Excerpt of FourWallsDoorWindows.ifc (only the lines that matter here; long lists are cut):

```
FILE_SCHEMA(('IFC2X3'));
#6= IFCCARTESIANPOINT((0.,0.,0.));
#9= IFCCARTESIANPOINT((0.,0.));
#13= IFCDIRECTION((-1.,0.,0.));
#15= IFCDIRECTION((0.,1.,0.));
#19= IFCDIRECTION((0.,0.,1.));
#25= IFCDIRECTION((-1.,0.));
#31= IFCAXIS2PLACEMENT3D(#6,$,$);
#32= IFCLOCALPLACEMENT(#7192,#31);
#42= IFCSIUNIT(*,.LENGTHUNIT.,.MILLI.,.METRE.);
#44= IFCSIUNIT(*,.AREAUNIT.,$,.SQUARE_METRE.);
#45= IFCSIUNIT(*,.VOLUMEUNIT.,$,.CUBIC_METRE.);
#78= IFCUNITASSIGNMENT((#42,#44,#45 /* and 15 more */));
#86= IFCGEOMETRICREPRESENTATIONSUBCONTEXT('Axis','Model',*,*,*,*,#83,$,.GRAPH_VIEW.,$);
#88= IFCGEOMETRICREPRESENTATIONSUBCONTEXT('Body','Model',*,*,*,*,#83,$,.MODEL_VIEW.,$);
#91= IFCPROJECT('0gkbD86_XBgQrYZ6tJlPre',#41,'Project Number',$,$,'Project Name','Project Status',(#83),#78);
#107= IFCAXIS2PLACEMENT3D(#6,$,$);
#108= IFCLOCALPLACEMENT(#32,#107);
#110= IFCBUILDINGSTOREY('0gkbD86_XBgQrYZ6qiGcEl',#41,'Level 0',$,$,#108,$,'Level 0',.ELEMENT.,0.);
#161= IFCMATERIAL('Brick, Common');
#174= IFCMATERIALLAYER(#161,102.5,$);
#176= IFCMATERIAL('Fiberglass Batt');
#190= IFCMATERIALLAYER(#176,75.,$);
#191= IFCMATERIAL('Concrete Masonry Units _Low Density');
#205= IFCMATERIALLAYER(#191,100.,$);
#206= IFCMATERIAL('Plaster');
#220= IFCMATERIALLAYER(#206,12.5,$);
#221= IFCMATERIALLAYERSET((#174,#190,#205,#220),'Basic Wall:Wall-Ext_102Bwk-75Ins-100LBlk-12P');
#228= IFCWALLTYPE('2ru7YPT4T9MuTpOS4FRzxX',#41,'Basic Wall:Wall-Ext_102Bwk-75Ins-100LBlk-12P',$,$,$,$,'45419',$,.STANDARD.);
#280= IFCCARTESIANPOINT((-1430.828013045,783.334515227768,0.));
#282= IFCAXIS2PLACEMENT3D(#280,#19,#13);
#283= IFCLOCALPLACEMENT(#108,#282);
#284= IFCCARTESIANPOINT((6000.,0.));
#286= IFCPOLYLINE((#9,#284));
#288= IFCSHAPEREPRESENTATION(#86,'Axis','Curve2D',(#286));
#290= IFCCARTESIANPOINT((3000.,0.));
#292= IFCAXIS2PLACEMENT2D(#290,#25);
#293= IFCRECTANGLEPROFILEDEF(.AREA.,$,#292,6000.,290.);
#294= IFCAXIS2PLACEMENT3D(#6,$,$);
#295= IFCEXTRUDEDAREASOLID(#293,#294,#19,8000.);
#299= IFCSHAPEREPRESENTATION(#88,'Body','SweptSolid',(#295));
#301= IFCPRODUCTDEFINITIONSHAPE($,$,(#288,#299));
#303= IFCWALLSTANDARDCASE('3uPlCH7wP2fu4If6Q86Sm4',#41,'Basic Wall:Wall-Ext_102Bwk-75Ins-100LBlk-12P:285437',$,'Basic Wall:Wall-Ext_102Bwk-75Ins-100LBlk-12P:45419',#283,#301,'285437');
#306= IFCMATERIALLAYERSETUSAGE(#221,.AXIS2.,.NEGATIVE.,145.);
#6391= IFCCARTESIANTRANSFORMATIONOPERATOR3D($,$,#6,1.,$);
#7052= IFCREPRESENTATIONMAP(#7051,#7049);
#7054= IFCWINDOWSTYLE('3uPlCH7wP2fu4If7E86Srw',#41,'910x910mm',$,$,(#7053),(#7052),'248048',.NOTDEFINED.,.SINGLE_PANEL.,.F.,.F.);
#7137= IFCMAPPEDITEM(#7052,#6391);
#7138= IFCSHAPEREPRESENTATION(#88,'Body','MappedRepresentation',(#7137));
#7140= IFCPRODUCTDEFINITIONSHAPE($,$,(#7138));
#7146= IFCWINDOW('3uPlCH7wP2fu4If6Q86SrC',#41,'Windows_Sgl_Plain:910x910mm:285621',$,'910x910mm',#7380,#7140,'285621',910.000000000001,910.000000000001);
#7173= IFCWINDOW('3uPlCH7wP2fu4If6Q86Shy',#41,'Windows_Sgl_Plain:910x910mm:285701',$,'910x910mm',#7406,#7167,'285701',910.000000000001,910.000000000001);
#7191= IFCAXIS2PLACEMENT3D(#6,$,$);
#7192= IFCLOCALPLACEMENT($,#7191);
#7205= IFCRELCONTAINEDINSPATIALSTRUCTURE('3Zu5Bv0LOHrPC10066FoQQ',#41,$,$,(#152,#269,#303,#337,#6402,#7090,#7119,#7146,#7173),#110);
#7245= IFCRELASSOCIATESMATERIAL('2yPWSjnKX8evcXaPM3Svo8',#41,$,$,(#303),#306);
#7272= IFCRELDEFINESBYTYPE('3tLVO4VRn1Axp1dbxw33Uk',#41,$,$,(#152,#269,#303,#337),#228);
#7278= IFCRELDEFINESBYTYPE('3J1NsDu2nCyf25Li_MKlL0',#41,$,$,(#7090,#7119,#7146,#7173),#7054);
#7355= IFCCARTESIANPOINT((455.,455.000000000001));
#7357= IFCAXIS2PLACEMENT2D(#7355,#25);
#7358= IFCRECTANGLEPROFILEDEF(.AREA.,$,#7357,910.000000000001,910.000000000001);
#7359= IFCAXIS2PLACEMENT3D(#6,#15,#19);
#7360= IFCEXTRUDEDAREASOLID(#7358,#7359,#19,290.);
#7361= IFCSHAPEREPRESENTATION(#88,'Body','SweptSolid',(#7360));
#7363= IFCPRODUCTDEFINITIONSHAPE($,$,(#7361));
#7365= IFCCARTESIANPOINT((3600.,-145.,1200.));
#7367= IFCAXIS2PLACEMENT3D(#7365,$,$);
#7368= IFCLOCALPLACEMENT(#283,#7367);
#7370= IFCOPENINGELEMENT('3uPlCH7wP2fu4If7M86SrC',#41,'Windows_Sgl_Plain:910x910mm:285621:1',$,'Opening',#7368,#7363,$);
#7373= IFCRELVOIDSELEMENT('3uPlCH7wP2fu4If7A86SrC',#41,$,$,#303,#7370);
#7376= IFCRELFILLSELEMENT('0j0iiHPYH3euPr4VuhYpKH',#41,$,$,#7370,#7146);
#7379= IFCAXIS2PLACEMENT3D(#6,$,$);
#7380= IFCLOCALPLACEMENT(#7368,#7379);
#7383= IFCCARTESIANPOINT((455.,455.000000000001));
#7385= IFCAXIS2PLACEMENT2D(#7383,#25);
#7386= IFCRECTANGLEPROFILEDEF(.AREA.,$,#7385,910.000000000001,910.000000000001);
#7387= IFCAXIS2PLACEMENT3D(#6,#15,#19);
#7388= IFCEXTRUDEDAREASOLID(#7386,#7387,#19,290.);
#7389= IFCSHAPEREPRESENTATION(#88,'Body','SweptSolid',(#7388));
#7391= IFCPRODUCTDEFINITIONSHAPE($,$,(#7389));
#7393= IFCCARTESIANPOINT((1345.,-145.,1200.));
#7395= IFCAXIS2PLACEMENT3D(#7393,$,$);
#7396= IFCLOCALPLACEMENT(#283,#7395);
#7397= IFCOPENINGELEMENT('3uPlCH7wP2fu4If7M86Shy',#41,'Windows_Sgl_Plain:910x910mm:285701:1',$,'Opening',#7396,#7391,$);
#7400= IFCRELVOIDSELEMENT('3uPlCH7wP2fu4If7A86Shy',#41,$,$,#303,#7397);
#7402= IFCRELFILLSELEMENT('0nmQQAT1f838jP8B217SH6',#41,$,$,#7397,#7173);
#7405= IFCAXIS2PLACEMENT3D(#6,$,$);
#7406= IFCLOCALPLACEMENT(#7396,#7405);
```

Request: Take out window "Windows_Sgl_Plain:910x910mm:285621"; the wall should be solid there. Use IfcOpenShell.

```python
import ifcopenshell
import ifcopenshell.api.feature
import ifcopenshell.api.root
import ifcopenshell.geom
import ifcopenshell.util.shape

model = ifcopenshell.open("FourWallsDoorWindows.ifc")
settings = ifcopenshell.geom.settings()


def volume(element):
    """Net volume in cubic metres, openings subtracted."""
    shape = ifcopenshell.geom.create_shape(settings, element)
    return ifcopenshell.util.shape.get_volume(shape.geometry)


window = model.by_guid("3uPlCH7wP2fu4If6Q86SrC")
opening = window.FillsVoids[0].RelatingOpeningElement
wall = opening.VoidsElements[0].RelatingBuildingElement
before = volume(wall)

ifcopenshell.api.root.remove_product(model, product=window)
ifcopenshell.api.feature.remove_feature(model, feature=opening)

after = volume(wall)

print(f"wall volume {before:.3f} -> {after:.3f} m3")

model.write("FourWallsDoorWindows_edited.ifc")
```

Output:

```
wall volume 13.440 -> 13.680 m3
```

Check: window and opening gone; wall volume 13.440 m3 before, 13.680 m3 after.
